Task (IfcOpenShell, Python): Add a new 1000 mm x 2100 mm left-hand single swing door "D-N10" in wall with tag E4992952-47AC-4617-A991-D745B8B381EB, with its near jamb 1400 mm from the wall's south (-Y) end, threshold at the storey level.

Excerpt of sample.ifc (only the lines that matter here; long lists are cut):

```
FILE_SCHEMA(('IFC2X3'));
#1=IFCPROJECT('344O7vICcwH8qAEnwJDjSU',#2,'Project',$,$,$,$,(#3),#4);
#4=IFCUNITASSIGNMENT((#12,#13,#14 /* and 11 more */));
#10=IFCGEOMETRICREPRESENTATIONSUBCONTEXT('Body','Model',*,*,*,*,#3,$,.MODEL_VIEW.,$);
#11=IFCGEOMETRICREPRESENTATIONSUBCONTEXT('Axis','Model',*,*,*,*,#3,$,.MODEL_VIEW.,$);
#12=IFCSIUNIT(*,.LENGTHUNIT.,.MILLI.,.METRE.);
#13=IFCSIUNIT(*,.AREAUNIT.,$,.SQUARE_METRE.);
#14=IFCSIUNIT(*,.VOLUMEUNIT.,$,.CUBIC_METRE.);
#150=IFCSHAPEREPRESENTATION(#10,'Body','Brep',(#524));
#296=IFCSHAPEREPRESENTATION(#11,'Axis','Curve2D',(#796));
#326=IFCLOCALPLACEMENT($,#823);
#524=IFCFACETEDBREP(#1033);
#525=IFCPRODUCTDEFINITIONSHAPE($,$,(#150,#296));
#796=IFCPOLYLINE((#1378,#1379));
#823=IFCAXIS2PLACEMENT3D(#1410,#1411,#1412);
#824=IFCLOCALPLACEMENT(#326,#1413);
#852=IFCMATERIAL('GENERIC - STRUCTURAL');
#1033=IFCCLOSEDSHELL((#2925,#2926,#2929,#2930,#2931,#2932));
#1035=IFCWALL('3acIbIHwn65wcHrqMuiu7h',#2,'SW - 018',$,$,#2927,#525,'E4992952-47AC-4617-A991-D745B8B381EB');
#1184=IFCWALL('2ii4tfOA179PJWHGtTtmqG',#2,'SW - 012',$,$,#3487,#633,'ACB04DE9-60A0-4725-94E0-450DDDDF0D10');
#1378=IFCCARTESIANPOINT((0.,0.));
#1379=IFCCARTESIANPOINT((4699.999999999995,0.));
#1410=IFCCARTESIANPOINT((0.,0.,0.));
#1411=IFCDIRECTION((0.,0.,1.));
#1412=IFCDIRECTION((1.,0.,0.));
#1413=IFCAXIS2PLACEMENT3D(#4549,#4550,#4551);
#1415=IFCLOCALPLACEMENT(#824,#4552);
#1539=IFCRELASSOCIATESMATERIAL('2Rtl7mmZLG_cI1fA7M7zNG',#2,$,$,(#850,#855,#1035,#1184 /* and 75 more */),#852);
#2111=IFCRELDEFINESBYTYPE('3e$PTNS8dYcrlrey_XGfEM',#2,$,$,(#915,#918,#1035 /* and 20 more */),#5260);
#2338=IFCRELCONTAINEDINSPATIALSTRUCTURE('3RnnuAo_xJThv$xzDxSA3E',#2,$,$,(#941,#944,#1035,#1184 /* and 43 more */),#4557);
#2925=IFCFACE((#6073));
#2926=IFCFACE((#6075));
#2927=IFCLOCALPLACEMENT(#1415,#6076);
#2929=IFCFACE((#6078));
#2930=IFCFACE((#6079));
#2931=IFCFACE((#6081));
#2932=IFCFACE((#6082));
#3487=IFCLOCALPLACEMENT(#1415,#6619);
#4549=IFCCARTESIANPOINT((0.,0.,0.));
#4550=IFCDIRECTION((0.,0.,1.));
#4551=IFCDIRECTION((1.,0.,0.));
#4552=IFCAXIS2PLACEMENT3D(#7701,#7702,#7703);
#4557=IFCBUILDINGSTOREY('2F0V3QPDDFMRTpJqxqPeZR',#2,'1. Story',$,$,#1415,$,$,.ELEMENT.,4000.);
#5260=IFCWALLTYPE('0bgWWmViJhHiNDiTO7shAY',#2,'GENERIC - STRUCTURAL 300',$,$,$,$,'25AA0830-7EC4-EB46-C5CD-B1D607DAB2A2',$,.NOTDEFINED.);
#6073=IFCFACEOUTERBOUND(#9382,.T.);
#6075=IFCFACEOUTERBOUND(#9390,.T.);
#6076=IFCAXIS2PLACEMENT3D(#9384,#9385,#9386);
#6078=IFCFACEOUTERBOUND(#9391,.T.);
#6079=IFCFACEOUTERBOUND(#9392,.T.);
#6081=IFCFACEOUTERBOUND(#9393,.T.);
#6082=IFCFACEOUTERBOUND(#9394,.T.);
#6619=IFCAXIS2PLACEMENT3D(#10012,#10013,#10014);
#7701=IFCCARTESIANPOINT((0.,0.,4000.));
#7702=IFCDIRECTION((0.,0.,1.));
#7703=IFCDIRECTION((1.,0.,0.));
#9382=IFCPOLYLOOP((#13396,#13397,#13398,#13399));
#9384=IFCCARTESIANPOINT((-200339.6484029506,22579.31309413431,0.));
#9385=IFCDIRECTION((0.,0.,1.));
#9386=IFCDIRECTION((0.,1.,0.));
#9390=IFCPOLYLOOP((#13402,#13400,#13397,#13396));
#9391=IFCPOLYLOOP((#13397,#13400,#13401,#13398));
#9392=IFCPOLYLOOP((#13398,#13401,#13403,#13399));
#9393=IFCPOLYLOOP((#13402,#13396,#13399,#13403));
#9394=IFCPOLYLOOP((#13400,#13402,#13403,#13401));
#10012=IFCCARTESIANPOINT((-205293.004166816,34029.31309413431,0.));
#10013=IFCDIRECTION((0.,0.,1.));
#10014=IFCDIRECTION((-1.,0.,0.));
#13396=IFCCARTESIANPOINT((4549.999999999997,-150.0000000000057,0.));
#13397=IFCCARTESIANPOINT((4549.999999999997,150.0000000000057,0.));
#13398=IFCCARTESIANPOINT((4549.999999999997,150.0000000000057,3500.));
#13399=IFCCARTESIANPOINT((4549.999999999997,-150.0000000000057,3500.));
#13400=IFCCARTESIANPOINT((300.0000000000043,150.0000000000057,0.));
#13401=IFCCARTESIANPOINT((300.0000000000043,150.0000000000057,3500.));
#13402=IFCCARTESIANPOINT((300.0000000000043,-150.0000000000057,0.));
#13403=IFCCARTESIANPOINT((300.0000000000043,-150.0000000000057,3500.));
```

```python
import numpy as np
import ifcopenshell
import ifcopenshell.api.feature
import ifcopenshell.api.geometry
import ifcopenshell.api.root
import ifcopenshell.api.spatial
import ifcopenshell.api.type
import ifcopenshell.geom
import ifcopenshell.util.element
import ifcopenshell.util.placement
import ifcopenshell.util.representation
import ifcopenshell.util.shape
import ifcopenshell.util.unit

model = ifcopenshell.open("sample.ifc")
unit_scale = ifcopenshell.util.unit.calculate_unit_scale(model)
settings = ifcopenshell.geom.settings()


def volume(element):
    """Net volume in cubic metres, openings subtracted."""
    shape = ifcopenshell.geom.create_shape(settings, element)
    return ifcopenshell.util.shape.get_volume(shape.geometry)


wall = model.by_guid("3acIbIHwn65wcHrqMuiu7h")
storey = ifcopenshell.util.element.get_container(wall, ifc_class="IfcBuildingStorey")
context = ifcopenshell.util.representation.get_context(model, "Model", "Body", "MODEL_VIEW")
before = volume(wall)

width, height, from_end, sill = 1, 2.1, 1.4, 0.0  # metres

# The wall runs along its own X axis, and the end named is its -X end.
wall_shape = ifcopenshell.geom.create_shape(settings, wall)
x, y, z = ifcopenshell.util.shape.get_vertices(wall_shape.geometry).T
start = x.min() + from_end
face, thickness = float(y.min()), float(y.max() - y.min())
wall_matrix = ifcopenshell.util.placement.get_local_placement(wall.ObjectPlacement)
level = ifcopenshell.util.placement.get_local_placement(storey.ObjectPlacement)[2, 3]


def in_wall(x, y):
    """Placement at x, y metres in the wall's axes, at sill height."""
    matrix = wall_matrix.copy()
    matrix[:, 3] = wall_matrix @ np.array([x / unit_scale, y / unit_scale, 0.0, 1.0])
    matrix[2, 3] = level + sill / unit_scale
    return matrix


# Opening: a box that overshoots both wall faces by 50 mm.
opening = ifcopenshell.api.root.create_entity(model, ifc_class="IfcOpeningElement")
box = ifcopenshell.api.geometry.add_wall_representation(
    model, context=context, length=width, height=height, thickness=thickness + 0.1
)
ifcopenshell.api.geometry.assign_representation(model, product=opening, representation=box)
ifcopenshell.api.geometry.edit_object_placement(model, product=opening, matrix=in_wall(start, face - 0.05), is_si=False)
ifcopenshell.api.feature.add_feature(model, feature=opening, element=wall)

door = ifcopenshell.api.root.create_entity(model, ifc_class="IfcDoor", name="D-N10")
door.OverallWidth, door.OverallHeight = width / unit_scale, height / unit_scale
body = ifcopenshell.api.geometry.add_door_representation(
    model,
    context=context,
    overall_width=door.OverallWidth,
    overall_height=door.OverallHeight,
    operation_type="SINGLE_SWING_LEFT",
    lining_properties={"LiningDepth": thickness / unit_scale, "ThresholdDepth": thickness / unit_scale},
)
ifcopenshell.api.geometry.assign_representation(model, product=door, representation=body)
ifcopenshell.api.spatial.assign_container(model, products=[door], relating_structure=storey)
fills = ifcopenshell.api.feature.add_filling(model, opening=opening, element=door)
fills.OwnerHistory = door.OwnerHistory  # required in IFC2X3

# IFC2X3 keeps the operation on the door style.
style = ifcopenshell.api.root.create_entity(model, ifc_class="IfcDoorStyle", name="D-N10")
style.OperationType, style.ConstructionType = "SINGLE_SWING_LEFT", "NOTDEFINED"
style.ParameterTakesPrecedence = style.Sizeable = False
ifcopenshell.api.type.assign_type(model, related_objects=[door], relating_type=style)

# The lining spans the wall, so the door starts at the wall face.
ifcopenshell.api.geometry.edit_object_placement(model, product=door, matrix=in_wall(start, face), is_si=False)

after = volume(wall)

print(f"wall volume {before:.3f} -> {after:.3f} m3")

model.write("sample_edited.ifc")
```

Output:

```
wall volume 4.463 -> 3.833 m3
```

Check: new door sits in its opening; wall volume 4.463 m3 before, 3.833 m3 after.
